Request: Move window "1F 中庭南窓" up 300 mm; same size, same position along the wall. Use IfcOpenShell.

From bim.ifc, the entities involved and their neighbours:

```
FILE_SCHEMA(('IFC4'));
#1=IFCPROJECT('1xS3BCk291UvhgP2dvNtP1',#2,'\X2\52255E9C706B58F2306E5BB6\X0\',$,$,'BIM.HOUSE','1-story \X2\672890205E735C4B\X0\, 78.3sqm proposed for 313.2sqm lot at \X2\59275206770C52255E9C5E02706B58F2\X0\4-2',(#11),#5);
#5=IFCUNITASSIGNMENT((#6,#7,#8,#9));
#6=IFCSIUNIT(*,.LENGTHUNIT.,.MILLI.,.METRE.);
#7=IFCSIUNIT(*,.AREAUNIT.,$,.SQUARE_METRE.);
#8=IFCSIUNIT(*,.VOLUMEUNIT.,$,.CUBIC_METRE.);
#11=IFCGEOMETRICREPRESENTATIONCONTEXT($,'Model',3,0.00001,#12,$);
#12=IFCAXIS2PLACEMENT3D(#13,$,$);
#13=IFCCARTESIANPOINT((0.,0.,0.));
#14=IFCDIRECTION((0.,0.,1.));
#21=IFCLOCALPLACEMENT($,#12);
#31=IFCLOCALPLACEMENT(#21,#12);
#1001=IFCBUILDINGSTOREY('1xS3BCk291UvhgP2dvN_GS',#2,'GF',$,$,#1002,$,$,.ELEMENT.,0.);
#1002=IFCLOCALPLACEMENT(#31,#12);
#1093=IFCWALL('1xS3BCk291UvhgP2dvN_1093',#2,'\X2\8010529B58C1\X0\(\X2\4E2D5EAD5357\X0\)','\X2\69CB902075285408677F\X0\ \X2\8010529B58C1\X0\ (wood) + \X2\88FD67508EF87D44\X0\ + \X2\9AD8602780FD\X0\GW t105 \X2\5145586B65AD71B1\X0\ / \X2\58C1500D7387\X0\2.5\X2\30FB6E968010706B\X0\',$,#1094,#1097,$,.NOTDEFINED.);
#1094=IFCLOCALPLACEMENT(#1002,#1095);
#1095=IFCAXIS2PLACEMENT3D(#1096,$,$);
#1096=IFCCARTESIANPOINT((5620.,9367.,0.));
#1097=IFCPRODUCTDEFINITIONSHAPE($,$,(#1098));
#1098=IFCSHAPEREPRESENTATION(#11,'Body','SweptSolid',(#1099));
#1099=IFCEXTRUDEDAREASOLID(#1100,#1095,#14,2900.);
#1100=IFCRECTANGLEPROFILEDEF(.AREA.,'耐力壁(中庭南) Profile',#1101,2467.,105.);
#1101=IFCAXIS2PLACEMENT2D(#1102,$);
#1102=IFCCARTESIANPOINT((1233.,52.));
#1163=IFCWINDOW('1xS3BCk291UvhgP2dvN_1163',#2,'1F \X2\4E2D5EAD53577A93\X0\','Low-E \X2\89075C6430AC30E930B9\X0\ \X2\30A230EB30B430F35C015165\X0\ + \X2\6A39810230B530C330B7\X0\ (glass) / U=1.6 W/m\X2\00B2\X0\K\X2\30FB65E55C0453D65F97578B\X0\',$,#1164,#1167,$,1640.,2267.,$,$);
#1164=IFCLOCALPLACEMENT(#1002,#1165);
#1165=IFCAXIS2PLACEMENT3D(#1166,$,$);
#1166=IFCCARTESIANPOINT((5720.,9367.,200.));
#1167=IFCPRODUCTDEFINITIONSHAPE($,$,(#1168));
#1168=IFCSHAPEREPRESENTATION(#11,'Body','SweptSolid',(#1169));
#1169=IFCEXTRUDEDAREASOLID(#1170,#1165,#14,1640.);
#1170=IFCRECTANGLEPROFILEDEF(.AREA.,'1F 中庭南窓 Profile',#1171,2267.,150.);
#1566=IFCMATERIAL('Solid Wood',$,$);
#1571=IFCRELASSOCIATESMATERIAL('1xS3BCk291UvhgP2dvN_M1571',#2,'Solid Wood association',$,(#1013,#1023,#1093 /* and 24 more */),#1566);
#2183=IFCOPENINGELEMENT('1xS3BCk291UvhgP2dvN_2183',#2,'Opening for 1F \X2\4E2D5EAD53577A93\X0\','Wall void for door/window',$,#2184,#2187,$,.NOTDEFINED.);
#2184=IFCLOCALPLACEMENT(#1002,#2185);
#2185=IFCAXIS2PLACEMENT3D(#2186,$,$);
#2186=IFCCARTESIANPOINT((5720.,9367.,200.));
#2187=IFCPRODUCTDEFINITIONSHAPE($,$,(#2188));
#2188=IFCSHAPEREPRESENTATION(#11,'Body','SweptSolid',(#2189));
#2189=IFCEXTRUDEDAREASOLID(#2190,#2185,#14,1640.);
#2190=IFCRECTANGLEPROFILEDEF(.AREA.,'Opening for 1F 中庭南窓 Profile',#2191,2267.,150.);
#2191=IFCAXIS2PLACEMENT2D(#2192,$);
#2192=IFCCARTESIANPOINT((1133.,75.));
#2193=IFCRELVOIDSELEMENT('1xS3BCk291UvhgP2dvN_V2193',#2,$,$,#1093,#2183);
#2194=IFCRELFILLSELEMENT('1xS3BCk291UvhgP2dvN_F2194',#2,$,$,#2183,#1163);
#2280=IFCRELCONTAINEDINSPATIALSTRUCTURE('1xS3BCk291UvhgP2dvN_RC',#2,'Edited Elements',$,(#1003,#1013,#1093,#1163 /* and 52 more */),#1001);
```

```python
import numpy as np
import ifcopenshell
import ifcopenshell.api.geometry
import ifcopenshell.util.placement
import ifcopenshell.util.unit

model = ifcopenshell.open("bim.ifc")
unit_scale = ifcopenshell.util.unit.calculate_unit_scale(model)

window = model.by_guid("1xS3BCk291UvhgP2dvN_1163")
opening = window.FillsVoids[0].RelatingOpeningElement
dz = 300.0

shift = np.array([0.0, 0.0, dz])
# The window is not placed relative to its opening, so move both.
for product in (opening, window):
    matrix = ifcopenshell.util.placement.get_local_placement(product.ObjectPlacement)
    matrix[:3, 3] += shift
    ifcopenshell.api.geometry.edit_object_placement(model, product=product, matrix=matrix, is_si=False)

print(f"moved by {dz * unit_scale:+.3f} m")

model.write("bim_rev.ifc")
```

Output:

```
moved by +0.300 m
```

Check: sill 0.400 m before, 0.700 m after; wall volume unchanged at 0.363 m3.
